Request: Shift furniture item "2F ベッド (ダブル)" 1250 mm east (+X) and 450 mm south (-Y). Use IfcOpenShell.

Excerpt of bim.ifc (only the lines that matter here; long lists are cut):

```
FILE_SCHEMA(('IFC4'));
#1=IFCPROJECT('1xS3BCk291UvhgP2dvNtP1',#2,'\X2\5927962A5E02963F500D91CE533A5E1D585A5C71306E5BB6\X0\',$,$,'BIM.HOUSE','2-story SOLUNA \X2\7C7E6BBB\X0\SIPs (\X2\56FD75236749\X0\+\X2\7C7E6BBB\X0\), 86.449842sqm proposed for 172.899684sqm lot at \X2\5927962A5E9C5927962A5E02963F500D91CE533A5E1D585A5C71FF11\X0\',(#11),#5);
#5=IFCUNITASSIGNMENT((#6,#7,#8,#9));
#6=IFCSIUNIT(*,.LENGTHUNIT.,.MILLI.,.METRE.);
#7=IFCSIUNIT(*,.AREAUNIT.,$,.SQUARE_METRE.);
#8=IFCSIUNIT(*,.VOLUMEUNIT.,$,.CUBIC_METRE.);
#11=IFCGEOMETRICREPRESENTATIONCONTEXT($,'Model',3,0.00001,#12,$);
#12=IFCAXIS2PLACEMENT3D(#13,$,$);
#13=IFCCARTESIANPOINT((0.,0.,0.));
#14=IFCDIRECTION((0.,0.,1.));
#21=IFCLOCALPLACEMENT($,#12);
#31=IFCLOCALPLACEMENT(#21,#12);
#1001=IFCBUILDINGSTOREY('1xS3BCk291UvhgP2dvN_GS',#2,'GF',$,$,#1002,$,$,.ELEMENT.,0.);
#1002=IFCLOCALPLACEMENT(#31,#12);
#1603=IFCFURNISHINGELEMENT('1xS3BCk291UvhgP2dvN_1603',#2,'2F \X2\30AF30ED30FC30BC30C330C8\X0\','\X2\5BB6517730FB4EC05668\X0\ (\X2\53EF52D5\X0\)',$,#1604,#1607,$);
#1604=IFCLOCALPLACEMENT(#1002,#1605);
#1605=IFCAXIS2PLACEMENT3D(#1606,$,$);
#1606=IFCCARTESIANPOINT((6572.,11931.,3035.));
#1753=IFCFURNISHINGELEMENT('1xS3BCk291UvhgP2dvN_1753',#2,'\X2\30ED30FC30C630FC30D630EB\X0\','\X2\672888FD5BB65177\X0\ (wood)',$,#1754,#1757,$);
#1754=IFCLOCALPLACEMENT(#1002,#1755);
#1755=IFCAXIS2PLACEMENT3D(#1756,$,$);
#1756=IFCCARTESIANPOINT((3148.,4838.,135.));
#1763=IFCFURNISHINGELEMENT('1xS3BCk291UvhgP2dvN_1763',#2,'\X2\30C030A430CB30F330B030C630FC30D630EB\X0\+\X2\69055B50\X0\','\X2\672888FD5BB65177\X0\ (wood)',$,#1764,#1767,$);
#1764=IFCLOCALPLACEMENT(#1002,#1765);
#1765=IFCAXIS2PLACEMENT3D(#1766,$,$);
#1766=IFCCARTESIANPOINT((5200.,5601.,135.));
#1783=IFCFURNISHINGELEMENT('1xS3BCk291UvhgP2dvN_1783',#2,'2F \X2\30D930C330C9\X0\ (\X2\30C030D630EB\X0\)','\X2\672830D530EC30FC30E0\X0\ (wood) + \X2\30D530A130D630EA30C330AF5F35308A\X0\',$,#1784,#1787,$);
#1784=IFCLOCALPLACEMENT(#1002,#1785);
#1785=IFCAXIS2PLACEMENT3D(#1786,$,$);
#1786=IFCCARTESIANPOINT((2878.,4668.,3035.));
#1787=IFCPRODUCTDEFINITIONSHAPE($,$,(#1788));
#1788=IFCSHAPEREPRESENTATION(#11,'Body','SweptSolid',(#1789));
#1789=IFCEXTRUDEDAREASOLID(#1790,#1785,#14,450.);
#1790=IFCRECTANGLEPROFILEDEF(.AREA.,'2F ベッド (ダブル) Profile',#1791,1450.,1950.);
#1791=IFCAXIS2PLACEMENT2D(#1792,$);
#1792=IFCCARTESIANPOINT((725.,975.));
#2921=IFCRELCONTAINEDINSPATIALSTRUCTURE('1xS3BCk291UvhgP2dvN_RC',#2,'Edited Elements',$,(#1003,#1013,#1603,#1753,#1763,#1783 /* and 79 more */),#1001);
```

```python
import ifcopenshell
import ifcopenshell.api.geometry
import ifcopenshell.util.placement
import ifcopenshell.util.unit

model = ifcopenshell.open("bim.ifc")
unit_scale = ifcopenshell.util.unit.calculate_unit_scale(model)

item = model.by_id(1783)
matrix = ifcopenshell.util.placement.get_local_placement(item.ObjectPlacement)
matrix[0, 3] += 1.25 / unit_scale
matrix[1, 3] -= 0.45 / unit_scale
ifcopenshell.api.geometry.edit_object_placement(model, product=item, matrix=matrix, is_si=False)

print(ifcopenshell.util.placement.get_local_placement(item.ObjectPlacement).round(3) + 0.0)

model.write("bim-out.ifc")
```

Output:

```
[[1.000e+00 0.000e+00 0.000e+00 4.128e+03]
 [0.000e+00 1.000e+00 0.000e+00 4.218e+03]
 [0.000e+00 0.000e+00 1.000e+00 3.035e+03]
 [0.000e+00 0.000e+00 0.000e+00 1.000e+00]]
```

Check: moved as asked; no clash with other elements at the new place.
